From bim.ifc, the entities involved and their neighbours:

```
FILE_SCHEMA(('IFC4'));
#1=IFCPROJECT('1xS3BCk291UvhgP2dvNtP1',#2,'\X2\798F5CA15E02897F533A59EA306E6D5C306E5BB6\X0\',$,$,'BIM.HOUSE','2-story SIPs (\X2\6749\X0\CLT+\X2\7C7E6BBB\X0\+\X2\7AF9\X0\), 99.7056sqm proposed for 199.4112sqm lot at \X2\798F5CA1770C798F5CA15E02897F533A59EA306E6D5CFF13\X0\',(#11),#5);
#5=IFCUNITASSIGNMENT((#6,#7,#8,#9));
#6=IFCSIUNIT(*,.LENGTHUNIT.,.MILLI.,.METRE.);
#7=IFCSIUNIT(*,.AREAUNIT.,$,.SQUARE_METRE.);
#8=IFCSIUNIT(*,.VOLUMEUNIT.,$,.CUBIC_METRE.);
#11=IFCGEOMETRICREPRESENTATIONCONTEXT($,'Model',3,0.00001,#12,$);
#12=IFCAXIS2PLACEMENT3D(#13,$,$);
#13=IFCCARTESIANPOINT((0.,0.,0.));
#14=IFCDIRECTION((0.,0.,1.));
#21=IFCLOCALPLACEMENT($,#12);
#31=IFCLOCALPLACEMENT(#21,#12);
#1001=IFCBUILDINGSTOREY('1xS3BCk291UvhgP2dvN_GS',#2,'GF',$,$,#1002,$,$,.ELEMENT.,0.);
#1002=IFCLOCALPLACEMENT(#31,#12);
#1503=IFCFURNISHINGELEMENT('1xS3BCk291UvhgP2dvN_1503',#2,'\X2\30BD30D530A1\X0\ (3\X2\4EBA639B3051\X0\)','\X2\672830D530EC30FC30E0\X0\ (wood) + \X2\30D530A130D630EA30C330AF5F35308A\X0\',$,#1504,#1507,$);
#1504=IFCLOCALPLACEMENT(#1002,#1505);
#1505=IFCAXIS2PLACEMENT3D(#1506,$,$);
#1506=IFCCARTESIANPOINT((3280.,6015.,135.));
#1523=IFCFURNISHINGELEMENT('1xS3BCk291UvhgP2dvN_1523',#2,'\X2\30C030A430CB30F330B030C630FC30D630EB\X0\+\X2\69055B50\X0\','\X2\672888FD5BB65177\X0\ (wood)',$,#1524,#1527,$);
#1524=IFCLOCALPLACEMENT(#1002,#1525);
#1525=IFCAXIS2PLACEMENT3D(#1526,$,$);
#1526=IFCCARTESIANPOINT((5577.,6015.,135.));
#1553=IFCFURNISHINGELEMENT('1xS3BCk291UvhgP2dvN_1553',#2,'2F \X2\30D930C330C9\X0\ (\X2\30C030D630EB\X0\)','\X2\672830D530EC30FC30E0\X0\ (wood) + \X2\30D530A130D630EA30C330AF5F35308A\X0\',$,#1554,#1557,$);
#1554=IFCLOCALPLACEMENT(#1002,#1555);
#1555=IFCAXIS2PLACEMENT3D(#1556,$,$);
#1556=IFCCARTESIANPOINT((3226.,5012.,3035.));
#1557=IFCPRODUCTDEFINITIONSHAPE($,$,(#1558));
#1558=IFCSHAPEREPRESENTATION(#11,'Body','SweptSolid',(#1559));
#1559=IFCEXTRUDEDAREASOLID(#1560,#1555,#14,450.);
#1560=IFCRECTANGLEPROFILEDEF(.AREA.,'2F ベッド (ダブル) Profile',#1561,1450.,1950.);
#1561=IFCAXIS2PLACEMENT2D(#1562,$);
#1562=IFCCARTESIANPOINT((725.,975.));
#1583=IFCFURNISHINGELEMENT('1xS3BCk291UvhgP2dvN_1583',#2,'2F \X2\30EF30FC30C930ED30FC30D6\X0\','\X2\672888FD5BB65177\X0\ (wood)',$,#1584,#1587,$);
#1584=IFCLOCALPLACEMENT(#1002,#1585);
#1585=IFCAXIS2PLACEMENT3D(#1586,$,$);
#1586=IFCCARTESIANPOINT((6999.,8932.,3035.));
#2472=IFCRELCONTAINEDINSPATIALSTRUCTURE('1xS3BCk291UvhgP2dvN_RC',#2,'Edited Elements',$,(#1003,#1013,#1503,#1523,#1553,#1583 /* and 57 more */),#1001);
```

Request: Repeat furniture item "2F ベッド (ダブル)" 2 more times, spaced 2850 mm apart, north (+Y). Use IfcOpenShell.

```python
import numpy as np
import ifcopenshell
import ifcopenshell.api.geometry
import ifcopenshell.api.root
import ifcopenshell.util.element
import ifcopenshell.util.placement

model = ifcopenshell.open("bim.ifc")


def reuse_history(source, copy):
    """copy_class also copies each property set's owner history, people and application; keep the originals."""
    for rel in copy.IsDefinedBy:
        if rel.is_a("IfcRelDefinesByProperties") and (history := rel.RelatingPropertyDefinition.OwnerHistory):
            rel.RelatingPropertyDefinition.OwnerHistory = source.OwnerHistory
            ifcopenshell.util.element.remove_deep2(model, history)


source = model.by_guid("1xS3BCk291UvhgP2dvN_1553")
base = ifcopenshell.util.placement.get_local_placement(source.ObjectPlacement)
step = np.array([0.0, 1.0, 0.0]) * 2850.0

for i in range(1, 3):
    copy = ifcopenshell.api.root.copy_class(model, product=source)
    copy.Representation = ifcopenshell.util.element.copy_deep(
        model, source.Representation, exclude=["IfcGeometricRepresentationContext", "IfcRepresentationMap"]
    )
    reuse_history(source, copy)
    matrix = base.copy()
    matrix[:3, 3] += i * step
    print("added at", matrix[:3, 3].round(3) + 0.0)
    ifcopenshell.api.geometry.edit_object_placement(model, product=copy, matrix=matrix, is_si=False)

model.write("bim_v2.ifc")
```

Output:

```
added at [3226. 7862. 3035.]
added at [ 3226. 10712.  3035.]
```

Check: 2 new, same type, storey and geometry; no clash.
